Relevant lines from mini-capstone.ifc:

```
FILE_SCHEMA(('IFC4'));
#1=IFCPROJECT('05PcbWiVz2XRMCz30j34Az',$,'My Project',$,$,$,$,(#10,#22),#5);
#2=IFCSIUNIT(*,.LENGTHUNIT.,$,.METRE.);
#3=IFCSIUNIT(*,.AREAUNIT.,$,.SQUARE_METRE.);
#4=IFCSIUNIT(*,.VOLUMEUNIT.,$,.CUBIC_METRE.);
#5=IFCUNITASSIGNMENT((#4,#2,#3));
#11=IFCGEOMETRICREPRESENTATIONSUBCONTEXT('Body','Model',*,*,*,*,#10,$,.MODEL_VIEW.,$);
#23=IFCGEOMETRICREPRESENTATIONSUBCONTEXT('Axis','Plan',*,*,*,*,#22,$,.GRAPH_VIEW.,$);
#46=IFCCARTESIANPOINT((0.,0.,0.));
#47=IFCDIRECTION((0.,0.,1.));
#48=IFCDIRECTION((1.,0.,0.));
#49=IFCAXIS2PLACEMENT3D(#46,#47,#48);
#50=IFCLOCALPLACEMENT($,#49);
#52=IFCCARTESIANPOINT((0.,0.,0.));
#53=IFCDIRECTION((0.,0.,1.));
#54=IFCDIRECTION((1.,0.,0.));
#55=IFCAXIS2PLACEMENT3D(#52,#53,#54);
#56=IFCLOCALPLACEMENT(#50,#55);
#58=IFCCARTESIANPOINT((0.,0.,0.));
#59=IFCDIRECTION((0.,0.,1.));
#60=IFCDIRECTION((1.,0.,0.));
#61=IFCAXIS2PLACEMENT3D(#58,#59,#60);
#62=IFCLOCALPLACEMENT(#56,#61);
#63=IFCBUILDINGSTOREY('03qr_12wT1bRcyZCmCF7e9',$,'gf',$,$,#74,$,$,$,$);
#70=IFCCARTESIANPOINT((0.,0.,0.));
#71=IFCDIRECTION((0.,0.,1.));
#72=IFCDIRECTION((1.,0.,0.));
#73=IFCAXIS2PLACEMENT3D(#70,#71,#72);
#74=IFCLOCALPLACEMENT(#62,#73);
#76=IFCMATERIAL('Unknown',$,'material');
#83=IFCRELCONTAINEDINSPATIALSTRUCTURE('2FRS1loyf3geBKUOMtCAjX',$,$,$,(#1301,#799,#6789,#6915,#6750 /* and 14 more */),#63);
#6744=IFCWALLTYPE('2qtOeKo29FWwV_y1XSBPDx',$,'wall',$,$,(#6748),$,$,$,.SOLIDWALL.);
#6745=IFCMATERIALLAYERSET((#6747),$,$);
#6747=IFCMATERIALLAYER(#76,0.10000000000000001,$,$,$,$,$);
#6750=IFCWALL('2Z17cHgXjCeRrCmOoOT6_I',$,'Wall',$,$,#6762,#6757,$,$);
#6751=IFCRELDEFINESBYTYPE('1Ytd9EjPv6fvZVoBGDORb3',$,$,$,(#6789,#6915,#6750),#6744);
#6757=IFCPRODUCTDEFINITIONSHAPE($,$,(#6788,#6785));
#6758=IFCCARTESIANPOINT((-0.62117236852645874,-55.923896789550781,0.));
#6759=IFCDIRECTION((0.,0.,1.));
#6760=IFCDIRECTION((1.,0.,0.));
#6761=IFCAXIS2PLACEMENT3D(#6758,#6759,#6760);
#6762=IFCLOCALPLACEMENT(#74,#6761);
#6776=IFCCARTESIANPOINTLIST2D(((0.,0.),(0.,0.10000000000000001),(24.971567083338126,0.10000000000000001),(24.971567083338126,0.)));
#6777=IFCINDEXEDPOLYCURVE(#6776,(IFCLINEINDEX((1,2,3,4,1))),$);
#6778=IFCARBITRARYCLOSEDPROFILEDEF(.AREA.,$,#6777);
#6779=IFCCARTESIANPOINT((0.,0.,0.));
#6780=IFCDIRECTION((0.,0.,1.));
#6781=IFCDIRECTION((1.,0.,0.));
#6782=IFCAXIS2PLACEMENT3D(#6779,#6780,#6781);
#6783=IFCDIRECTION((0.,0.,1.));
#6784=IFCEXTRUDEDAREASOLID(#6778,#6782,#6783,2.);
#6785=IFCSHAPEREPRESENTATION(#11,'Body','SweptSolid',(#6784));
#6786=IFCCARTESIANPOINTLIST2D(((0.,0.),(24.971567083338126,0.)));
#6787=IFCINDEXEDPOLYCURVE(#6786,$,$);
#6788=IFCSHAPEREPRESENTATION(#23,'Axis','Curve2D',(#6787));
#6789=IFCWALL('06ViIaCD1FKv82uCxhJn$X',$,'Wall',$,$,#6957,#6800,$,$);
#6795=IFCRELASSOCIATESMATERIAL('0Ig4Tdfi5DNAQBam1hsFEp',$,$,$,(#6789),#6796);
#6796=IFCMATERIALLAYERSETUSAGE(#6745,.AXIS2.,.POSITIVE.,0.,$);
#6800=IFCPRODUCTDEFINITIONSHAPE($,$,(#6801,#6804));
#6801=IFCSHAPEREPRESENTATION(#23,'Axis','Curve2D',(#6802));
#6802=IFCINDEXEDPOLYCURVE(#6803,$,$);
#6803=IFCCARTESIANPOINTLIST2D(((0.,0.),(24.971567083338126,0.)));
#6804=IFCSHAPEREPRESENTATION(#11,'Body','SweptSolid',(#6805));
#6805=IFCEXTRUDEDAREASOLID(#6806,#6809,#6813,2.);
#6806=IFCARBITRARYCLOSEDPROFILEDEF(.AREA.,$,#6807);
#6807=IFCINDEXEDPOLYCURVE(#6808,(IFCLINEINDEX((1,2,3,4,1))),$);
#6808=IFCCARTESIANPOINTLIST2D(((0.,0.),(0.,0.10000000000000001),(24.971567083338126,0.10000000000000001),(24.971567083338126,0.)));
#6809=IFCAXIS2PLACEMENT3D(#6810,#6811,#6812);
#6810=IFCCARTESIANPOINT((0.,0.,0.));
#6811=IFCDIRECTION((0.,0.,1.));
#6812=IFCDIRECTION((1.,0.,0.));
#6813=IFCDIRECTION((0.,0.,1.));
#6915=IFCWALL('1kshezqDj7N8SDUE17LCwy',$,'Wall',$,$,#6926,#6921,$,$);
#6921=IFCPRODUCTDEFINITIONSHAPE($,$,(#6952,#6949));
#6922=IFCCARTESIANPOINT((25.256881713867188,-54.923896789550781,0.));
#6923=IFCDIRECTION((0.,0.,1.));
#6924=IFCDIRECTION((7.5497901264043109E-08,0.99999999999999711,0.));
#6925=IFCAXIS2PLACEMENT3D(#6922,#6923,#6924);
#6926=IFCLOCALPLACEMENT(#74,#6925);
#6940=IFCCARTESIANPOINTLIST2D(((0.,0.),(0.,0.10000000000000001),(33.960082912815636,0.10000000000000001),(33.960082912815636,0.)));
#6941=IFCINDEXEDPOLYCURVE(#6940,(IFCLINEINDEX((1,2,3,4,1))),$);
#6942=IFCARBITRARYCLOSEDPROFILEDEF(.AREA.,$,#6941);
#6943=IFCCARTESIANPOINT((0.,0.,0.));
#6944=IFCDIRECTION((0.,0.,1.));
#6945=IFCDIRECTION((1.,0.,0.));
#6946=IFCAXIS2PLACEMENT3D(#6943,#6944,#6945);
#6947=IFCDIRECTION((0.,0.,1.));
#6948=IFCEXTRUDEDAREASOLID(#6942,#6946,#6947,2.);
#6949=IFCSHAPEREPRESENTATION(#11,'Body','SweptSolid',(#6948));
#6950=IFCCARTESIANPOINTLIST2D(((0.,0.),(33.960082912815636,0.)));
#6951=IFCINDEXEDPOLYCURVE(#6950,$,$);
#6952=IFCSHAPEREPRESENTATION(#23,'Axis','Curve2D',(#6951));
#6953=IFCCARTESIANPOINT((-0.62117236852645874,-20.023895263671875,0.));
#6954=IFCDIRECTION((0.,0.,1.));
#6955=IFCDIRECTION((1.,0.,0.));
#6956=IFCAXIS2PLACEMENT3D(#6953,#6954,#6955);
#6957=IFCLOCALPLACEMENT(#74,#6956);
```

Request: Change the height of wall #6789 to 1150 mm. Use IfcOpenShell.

```python
import ifcopenshell
import ifcopenshell.geom
import ifcopenshell.util.representation
import ifcopenshell.util.shape

model = ifcopenshell.open("mini-capstone.ifc")
settings = ifcopenshell.geom.settings()


def volume(element):
    """Net volume in cubic metres, openings subtracted."""
    shape = ifcopenshell.geom.create_shape(settings, element)
    return ifcopenshell.util.shape.get_volume(shape.geometry)


wall = model.by_guid("06ViIaCD1FKv82uCxhJn$X")
before = volume(wall)

body = ifcopenshell.util.representation.get_representation(wall, "Model", "Body")
solid = body.Items[0]
old_height = solid.Depth
solid.Depth = 1.15
after = volume(wall)

print(f"height {old_height:g} -> {solid.Depth:g}, volume {before:.3f} -> {after:.3f} m3")

model.write("mini-capstone_v2.ifc")
```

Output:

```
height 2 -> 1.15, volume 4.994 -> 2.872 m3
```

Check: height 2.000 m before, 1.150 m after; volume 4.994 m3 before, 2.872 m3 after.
